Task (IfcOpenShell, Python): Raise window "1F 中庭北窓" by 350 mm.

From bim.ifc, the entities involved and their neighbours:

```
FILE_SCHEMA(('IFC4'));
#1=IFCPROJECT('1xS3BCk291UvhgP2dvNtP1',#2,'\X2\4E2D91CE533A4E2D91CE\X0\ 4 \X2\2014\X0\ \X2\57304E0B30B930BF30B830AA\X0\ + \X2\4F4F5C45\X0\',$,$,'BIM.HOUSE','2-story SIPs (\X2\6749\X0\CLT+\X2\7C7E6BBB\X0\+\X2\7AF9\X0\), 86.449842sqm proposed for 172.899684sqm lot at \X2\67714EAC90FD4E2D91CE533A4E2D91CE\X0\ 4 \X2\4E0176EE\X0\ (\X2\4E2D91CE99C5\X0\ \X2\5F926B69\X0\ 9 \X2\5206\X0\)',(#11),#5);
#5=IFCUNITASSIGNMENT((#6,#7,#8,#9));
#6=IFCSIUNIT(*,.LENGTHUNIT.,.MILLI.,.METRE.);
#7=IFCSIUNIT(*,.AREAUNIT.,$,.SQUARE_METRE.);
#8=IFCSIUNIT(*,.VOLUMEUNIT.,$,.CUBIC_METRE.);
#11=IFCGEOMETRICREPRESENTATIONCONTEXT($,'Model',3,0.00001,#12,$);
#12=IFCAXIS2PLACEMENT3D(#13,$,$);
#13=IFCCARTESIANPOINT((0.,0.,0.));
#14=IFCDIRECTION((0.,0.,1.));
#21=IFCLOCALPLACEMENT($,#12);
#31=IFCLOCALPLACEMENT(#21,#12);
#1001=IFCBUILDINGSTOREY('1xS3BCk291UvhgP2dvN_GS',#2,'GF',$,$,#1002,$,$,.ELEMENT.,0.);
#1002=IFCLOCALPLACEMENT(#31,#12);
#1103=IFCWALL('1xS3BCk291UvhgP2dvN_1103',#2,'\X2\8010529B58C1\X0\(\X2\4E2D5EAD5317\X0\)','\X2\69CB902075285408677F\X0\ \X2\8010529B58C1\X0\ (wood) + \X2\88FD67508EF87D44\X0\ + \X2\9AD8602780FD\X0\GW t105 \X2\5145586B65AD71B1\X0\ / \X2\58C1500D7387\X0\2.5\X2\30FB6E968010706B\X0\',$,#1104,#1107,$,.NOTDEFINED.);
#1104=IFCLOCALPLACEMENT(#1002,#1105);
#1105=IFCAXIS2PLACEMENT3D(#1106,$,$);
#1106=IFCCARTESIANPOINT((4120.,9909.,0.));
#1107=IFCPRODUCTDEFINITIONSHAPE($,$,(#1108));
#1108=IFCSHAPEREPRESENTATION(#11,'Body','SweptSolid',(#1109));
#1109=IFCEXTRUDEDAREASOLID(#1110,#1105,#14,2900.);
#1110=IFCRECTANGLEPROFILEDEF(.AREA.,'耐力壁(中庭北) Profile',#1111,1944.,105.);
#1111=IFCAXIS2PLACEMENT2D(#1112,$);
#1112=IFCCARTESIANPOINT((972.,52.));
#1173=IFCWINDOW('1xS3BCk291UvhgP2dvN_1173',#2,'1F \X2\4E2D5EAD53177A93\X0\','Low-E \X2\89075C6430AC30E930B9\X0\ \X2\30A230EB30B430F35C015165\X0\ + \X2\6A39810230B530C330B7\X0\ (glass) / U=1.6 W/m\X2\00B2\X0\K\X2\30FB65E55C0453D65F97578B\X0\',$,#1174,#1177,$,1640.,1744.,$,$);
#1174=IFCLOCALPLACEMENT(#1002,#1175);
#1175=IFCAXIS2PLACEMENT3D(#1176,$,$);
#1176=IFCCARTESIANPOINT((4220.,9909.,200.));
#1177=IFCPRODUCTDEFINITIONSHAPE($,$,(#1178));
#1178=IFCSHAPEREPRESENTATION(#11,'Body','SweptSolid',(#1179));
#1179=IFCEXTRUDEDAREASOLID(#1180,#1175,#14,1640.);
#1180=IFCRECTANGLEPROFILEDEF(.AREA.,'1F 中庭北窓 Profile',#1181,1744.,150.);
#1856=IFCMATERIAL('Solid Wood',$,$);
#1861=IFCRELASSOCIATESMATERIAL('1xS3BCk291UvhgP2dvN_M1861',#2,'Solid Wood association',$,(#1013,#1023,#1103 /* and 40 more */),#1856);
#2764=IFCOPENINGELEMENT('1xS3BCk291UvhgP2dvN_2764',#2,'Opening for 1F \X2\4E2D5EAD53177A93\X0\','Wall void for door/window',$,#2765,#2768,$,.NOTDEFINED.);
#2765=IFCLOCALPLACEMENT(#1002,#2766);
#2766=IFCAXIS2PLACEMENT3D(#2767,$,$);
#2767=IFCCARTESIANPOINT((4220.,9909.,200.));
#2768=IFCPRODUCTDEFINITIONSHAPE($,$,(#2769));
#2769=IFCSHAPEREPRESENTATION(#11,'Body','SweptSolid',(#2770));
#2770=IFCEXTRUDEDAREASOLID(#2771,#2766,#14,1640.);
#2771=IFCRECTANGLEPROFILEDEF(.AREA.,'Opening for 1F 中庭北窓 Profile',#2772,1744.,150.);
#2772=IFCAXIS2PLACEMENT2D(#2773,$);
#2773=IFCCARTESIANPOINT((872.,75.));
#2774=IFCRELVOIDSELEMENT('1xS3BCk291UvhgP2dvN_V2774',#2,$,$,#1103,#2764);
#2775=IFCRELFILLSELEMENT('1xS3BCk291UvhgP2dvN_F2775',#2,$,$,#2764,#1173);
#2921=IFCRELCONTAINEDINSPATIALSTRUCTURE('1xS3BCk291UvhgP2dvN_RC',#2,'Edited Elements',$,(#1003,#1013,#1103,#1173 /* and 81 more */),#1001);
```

```python
import numpy as np
import ifcopenshell
import ifcopenshell.api.geometry
import ifcopenshell.util.placement
import ifcopenshell.util.unit

model = ifcopenshell.open("bim.ifc")
unit_scale = ifcopenshell.util.unit.calculate_unit_scale(model)

window = model.by_guid("1xS3BCk291UvhgP2dvN_1173")
opening = window.FillsVoids[0].RelatingOpeningElement
dz = 0.35 / unit_scale

shift = np.array([0.0, 0.0, dz])
# The window is not placed relative to its opening, so move both.
for product in (opening, window):
    matrix = ifcopenshell.util.placement.get_local_placement(product.ObjectPlacement)
    matrix[:3, 3] += shift
    ifcopenshell.api.geometry.edit_object_placement(model, product=product, matrix=matrix, is_si=False)

print(f"moved by {dz * unit_scale:+.3f} m")

model.write("bim_v2.ifc")
```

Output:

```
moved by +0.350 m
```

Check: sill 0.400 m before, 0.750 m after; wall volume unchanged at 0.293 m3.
